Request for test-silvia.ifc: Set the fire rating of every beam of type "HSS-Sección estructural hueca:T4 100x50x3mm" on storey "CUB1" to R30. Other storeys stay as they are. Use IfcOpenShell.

First a look at what the model holds.

```python
import ifcopenshell
import ifcopenshell.util.element

model = ifcopenshell.open("test-silvia.ifc")
print(model.schema)
storey = next(s for s in model.by_type("IfcBuildingStorey") if s.Name == "CUB1")
beams = [e for e in ifcopenshell.util.element.get_decomposition(storey) if e.is_a("IfcBeam")]
seen = {}
for e in beams:
    element_type = ifcopenshell.util.element.get_type(e)
    key = (element_type.Name if element_type != e and element_type else None, ifcopenshell.util.element.get_pset(e, "Pset_BeamCommon", "FireRating"))
    seen[key] = seen.get(key, 0) + 1
for (name, value), count in sorted(seen.items(), key=str):
    print(count, "x", name, "|", value)
```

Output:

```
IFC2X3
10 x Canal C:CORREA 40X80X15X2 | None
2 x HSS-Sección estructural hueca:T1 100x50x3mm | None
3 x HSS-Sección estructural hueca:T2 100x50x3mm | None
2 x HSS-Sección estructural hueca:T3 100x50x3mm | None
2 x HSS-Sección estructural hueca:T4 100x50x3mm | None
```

```python
import ifcopenshell
import ifcopenshell.api.pset
import ifcopenshell.util.element

model = ifcopenshell.open("test-silvia.ifc")

storey = next(s for s in model.by_type("IfcBuildingStorey") if s.Name == "CUB1")
beams = [e for e in ifcopenshell.util.element.get_decomposition(storey) if e.is_a("IfcBeam")]

count = 0
for e in beams:
    element_type = ifcopenshell.util.element.get_type(e)
    if element_type in (None, e) or element_type.Name != "HSS-Sección estructural hueca:T4 100x50x3mm":
        continue
    # add_pset returns the element's existing set when there is one.
    pset = ifcopenshell.api.pset.add_pset(model, product=e, name="Pset_BeamCommon")
    ifcopenshell.api.pset.edit_pset(model, pset=pset, properties={"FireRating": "R30"})
    count += 1

print(count, "beams updated")

model.write("test-silvia_updated.ifc")
```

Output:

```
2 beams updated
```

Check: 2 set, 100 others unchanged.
